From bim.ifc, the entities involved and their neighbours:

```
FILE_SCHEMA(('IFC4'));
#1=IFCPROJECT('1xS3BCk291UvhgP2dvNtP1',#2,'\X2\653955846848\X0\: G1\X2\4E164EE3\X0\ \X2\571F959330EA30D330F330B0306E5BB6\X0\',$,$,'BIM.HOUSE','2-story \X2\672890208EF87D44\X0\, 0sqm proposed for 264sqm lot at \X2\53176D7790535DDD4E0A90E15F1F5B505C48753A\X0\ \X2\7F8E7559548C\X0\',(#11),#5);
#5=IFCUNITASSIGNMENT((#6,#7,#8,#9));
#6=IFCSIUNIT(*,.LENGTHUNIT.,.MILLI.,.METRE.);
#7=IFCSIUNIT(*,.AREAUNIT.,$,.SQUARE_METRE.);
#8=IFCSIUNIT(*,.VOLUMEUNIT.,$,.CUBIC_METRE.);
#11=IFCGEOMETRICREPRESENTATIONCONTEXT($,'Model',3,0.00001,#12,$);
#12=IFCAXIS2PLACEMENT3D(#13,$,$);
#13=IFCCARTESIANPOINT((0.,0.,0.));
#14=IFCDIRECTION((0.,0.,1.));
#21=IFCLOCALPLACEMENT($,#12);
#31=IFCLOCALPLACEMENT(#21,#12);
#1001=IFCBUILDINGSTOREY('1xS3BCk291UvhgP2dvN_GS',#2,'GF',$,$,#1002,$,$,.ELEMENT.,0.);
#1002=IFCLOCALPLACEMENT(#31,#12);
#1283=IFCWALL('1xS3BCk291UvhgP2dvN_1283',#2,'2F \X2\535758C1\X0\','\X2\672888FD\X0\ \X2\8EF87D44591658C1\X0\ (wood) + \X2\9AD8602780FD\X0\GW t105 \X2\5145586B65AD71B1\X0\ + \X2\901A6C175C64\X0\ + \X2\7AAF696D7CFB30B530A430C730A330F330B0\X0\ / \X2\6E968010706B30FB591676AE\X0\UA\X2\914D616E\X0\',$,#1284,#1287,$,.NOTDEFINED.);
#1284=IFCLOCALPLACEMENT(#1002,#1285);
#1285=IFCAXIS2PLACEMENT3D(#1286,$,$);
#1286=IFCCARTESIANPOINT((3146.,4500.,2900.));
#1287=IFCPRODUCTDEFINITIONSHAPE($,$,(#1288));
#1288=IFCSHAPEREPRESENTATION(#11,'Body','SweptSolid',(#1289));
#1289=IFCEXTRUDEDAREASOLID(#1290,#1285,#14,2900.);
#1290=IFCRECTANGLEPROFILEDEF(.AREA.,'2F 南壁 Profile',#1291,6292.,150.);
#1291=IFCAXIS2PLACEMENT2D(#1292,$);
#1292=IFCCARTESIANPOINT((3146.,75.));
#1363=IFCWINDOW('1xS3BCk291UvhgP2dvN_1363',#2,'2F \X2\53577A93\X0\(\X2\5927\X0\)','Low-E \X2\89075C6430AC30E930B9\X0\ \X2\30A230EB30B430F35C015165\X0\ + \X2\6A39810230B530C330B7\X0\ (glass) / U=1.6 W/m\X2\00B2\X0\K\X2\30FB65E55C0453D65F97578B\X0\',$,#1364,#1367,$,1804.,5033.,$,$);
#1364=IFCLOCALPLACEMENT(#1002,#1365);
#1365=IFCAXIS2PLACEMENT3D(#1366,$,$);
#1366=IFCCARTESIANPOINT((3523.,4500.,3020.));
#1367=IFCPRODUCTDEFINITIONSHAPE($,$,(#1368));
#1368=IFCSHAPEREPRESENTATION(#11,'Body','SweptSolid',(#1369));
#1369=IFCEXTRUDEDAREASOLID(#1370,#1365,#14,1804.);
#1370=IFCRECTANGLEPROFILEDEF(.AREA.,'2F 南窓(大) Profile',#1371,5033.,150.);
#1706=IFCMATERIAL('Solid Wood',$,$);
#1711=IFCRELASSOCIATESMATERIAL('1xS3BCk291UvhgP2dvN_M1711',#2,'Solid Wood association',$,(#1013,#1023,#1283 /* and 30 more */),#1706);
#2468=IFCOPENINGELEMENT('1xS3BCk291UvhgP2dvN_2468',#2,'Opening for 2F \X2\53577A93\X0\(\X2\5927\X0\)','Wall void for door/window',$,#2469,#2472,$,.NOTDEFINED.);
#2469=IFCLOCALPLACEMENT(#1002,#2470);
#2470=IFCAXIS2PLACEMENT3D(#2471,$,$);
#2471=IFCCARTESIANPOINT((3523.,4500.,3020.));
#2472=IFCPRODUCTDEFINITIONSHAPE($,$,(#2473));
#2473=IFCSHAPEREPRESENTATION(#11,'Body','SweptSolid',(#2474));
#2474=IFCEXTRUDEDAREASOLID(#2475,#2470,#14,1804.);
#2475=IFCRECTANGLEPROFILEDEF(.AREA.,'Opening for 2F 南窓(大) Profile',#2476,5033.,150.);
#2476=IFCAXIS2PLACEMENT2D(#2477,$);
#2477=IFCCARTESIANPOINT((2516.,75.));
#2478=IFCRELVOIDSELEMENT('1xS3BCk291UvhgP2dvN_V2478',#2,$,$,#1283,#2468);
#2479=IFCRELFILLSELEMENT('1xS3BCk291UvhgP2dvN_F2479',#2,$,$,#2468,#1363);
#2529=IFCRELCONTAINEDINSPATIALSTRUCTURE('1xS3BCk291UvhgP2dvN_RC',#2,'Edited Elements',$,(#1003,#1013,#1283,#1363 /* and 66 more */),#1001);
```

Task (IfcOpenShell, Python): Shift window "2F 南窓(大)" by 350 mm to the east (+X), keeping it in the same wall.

```python
import ifcopenshell
import ifcopenshell.api.geometry
import ifcopenshell.util.placement

model = ifcopenshell.open("bim.ifc")

window = model.by_guid("1xS3BCk291UvhgP2dvN_1363")
opening = window.FillsVoids[0].RelatingOpeningElement
wall = opening.VoidsElements[0].RelatingBuildingElement

wall_matrix = ifcopenshell.util.placement.get_local_placement(wall.ObjectPlacement)
shift = wall_matrix[:3, 0] * 350.0
before = ifcopenshell.util.placement.get_local_placement(window.ObjectPlacement)[:3, 3].copy()

# The window is not placed relative to its opening, so move both.
for product in (opening, window):
    matrix = ifcopenshell.util.placement.get_local_placement(product.ObjectPlacement)
    matrix[:3, 3] += shift
    ifcopenshell.api.geometry.edit_object_placement(model, product=product, matrix=matrix, is_si=False)

after = ifcopenshell.util.placement.get_local_placement(window.ObjectPlacement)[:3, 3]
print("window moved by", (after - before).round(3) + 0.0)

model.write("bim_rev.ifc")
```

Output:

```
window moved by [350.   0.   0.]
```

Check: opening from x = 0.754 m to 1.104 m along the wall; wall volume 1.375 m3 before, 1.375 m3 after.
